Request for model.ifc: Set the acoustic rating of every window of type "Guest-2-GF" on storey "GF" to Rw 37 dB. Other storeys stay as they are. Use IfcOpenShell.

First a look at what the model holds.

```python
import ifcopenshell
import ifcopenshell.util.element

model = ifcopenshell.open("model.ifc")
print(model.schema)
storey = next(s for s in model.by_type("IfcBuildingStorey") if s.Name == "GF")
windows = [e for e in ifcopenshell.util.element.get_decomposition(storey) if e.is_a("IfcWindow")]
seen = {}
for e in windows:
    element_type = ifcopenshell.util.element.get_type(e)
    key = (element_type.Name if element_type != e and element_type else None, ifcopenshell.util.element.get_pset(e, "Pset_WindowCommon", "AcousticRating"))
    seen[key] = seen.get(key, 0) + 1
for (name, value), count in sorted(seen.items(), key=str):
    print(count, "x", name, "|", value)
```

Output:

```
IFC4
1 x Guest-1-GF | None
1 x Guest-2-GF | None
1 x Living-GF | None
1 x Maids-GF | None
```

```python
import ifcopenshell
import ifcopenshell.api.pset
import ifcopenshell.util.element

model = ifcopenshell.open("model.ifc")

storey = next(s for s in model.by_type("IfcBuildingStorey") if s.Name == "GF")
windows = [e for e in ifcopenshell.util.element.get_decomposition(storey) if e.is_a("IfcWindow")]

count = 0
for e in windows:
    element_type = ifcopenshell.util.element.get_type(e)
    if element_type in (None, e) or element_type.Name != "Guest-2-GF":
        continue
    # add_pset returns the element's existing set when there is one.
    pset = ifcopenshell.api.pset.add_pset(model, product=e, name="Pset_WindowCommon")
    ifcopenshell.api.pset.edit_pset(model, pset=pset, properties={"AcousticRating": "Rw 37 dB"})
    count += 1

print(count, "windows updated")

model.write("model-out.ifc")
```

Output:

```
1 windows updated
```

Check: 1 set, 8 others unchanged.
